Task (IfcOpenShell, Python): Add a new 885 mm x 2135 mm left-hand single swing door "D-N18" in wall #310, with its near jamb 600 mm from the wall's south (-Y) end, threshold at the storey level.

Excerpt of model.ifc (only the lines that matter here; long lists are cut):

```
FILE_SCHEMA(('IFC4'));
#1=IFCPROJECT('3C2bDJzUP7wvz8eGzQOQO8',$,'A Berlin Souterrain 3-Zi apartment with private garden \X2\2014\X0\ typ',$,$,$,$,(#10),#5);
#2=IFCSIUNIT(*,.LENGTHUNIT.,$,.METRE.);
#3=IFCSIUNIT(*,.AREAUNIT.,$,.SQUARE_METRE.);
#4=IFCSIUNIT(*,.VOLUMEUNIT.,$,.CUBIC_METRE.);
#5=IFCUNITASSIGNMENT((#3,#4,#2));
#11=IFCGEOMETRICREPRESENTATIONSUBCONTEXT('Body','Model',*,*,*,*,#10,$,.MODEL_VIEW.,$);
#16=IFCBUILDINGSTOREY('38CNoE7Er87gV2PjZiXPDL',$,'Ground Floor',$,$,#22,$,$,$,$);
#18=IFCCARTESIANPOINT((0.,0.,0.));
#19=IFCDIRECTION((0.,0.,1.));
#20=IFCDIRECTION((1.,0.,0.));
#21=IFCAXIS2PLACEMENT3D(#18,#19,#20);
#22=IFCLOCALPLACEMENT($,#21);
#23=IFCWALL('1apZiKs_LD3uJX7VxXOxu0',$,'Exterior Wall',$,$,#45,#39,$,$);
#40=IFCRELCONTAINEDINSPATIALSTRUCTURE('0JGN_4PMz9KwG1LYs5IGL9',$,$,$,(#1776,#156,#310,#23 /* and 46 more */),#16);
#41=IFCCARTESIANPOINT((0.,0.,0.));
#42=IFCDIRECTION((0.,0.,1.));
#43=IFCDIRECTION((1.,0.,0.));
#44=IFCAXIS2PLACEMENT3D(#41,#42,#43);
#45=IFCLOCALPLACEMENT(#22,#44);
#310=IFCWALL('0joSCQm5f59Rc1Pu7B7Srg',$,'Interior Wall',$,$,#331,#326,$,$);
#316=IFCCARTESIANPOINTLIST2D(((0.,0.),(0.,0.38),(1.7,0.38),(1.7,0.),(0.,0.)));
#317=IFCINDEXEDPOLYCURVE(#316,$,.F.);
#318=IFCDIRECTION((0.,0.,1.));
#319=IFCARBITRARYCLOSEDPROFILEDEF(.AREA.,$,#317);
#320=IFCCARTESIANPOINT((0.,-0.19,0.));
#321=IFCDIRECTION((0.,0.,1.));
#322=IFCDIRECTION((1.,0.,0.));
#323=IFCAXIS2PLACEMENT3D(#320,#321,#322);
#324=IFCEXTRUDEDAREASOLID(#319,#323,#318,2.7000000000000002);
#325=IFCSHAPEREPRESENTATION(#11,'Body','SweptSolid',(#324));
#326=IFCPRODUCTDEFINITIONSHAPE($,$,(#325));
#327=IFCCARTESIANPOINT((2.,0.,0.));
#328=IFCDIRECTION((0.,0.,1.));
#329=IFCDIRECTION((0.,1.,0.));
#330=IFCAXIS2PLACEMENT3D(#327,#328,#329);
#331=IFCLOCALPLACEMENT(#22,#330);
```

```python
import numpy as np
import ifcopenshell
import ifcopenshell.api.feature
import ifcopenshell.api.geometry
import ifcopenshell.api.root
import ifcopenshell.api.spatial
import ifcopenshell.geom
import ifcopenshell.util.element
import ifcopenshell.util.placement
import ifcopenshell.util.representation
import ifcopenshell.util.shape
import ifcopenshell.util.unit

model = ifcopenshell.open("model.ifc")
unit_scale = ifcopenshell.util.unit.calculate_unit_scale(model)
settings = ifcopenshell.geom.settings()


def volume(element):
    """Net volume in cubic metres, openings subtracted."""
    shape = ifcopenshell.geom.create_shape(settings, element)
    return ifcopenshell.util.shape.get_volume(shape.geometry)


wall = model.by_id(310)
storey = ifcopenshell.util.element.get_container(wall, ifc_class="IfcBuildingStorey")
context = ifcopenshell.util.representation.get_context(model, "Model", "Body", "MODEL_VIEW")
before = volume(wall)

width, height, from_end, sill = 0.885, 2.135, 0.6, 0.0  # metres

# The wall runs along its own X axis, and the end named is its -X end.
wall_shape = ifcopenshell.geom.create_shape(settings, wall)
x, y, z = ifcopenshell.util.shape.get_vertices(wall_shape.geometry).T
start = x.min() + from_end
face, thickness = float(y.min()), float(y.max() - y.min())
wall_matrix = ifcopenshell.util.placement.get_local_placement(wall.ObjectPlacement)
level = ifcopenshell.util.placement.get_local_placement(storey.ObjectPlacement)[2, 3]


def in_wall(x, y):
    """Placement at x, y metres in the wall's axes, at sill height."""
    matrix = wall_matrix.copy()
    matrix[:, 3] = wall_matrix @ np.array([x / unit_scale, y / unit_scale, 0.0, 1.0])
    matrix[2, 3] = level + sill / unit_scale
    return matrix


# Opening: a box that overshoots both wall faces by 50 mm.
opening = ifcopenshell.api.root.create_entity(model, ifc_class="IfcOpeningElement", predefined_type="OPENING")
box = ifcopenshell.api.geometry.add_wall_representation(
    model, context=context, length=width, height=height, thickness=thickness + 0.1
)
ifcopenshell.api.geometry.assign_representation(model, product=opening, representation=box)
ifcopenshell.api.geometry.edit_object_placement(model, product=opening, matrix=in_wall(start, face - 0.05), is_si=False)
ifcopenshell.api.feature.add_feature(model, feature=opening, element=wall)

door = ifcopenshell.api.root.create_entity(model, ifc_class="IfcDoor", name="D-N18", predefined_type="DOOR")
door.OverallWidth, door.OverallHeight = width / unit_scale, height / unit_scale
door.OperationType = "SINGLE_SWING_LEFT"
body = ifcopenshell.api.geometry.add_door_representation(
    model,
    context=context,
    overall_width=door.OverallWidth,
    overall_height=door.OverallHeight,
    operation_type="SINGLE_SWING_LEFT",
    lining_properties={"LiningDepth": thickness / unit_scale, "ThresholdDepth": thickness / unit_scale},
)
ifcopenshell.api.geometry.assign_representation(model, product=door, representation=body)
ifcopenshell.api.spatial.assign_container(model, products=[door], relating_structure=storey)
ifcopenshell.api.feature.add_filling(model, opening=opening, element=door)

# The lining spans the wall, so the door starts at the wall face.
ifcopenshell.api.geometry.edit_object_placement(model, product=door, matrix=in_wall(start, face), is_si=False)

after = volume(wall)

print(f"wall volume {before:.3f} -> {after:.3f} m3")

model.write("model_rev.ifc")
```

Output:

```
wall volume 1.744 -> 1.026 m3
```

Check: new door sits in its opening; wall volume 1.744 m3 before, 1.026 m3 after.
